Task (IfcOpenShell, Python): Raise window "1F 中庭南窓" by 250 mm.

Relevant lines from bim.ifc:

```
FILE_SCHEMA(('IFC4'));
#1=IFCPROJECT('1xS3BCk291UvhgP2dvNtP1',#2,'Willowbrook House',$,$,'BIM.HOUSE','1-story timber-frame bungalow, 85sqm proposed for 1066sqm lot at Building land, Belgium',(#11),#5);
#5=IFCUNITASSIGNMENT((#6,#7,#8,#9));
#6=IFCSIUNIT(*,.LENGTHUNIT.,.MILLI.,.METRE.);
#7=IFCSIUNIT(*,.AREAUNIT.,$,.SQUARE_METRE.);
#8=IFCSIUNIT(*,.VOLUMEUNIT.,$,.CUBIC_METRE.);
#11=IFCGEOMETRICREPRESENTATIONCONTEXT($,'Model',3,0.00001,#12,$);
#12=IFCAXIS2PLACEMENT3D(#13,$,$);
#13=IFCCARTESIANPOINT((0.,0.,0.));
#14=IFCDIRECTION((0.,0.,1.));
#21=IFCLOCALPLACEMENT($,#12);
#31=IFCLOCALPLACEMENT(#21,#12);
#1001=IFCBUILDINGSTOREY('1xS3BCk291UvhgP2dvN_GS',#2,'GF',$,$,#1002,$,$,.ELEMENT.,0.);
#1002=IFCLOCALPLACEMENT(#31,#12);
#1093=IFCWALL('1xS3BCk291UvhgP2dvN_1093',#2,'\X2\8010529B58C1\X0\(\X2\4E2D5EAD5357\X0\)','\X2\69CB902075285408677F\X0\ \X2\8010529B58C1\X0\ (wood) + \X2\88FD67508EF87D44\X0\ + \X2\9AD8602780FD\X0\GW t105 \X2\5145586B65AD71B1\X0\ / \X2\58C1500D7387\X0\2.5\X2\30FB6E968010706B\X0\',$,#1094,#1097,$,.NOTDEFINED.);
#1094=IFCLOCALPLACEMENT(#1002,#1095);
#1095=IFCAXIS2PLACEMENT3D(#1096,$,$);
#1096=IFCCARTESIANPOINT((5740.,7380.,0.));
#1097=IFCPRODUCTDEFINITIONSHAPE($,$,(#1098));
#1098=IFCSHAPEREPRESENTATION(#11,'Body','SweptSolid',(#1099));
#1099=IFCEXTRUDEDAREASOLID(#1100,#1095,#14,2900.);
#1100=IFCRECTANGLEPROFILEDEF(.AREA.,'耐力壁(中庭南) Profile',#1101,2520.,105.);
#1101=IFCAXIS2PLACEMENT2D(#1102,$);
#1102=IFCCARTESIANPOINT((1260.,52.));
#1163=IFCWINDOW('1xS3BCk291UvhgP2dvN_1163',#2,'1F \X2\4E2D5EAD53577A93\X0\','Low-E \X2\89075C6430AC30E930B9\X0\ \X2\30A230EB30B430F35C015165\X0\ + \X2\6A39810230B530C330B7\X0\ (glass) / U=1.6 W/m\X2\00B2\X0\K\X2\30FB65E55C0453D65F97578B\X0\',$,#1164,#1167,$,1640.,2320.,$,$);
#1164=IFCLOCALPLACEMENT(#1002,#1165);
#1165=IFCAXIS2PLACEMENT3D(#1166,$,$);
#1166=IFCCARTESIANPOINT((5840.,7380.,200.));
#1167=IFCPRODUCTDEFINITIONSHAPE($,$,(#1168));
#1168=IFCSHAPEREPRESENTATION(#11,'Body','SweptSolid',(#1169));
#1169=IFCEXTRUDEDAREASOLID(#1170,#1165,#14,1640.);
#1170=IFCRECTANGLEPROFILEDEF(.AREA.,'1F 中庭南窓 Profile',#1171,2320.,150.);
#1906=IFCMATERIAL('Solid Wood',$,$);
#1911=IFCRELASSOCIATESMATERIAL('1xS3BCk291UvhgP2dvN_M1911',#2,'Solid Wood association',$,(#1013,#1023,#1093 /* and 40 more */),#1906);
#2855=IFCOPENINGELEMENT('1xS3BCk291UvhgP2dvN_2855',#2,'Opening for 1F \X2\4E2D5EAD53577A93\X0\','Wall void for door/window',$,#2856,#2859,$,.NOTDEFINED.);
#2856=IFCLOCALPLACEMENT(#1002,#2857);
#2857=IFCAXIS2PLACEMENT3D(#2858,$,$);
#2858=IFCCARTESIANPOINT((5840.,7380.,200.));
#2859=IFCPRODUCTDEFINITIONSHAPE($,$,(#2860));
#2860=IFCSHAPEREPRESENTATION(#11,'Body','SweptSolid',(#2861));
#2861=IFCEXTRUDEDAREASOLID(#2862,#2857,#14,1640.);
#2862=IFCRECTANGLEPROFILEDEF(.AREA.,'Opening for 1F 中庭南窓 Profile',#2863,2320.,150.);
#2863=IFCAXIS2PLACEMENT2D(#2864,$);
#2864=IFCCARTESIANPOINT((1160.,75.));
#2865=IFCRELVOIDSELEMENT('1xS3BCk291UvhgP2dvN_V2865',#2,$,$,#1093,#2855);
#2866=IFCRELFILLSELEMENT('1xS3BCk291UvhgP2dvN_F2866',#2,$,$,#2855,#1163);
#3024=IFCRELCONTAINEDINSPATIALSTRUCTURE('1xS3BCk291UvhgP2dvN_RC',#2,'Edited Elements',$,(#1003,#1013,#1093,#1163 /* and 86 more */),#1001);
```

```python
import numpy as np
import ifcopenshell
import ifcopenshell.api.geometry
import ifcopenshell.util.placement
import ifcopenshell.util.unit

model = ifcopenshell.open("bim.ifc")
unit_scale = ifcopenshell.util.unit.calculate_unit_scale(model)

window = model.by_guid("1xS3BCk291UvhgP2dvN_1163")
opening = window.FillsVoids[0].RelatingOpeningElement
dz = 250.0

shift = np.array([0.0, 0.0, dz])
# The window is not placed relative to its opening, so move both.
for product in (opening, window):
    matrix = ifcopenshell.util.placement.get_local_placement(product.ObjectPlacement)
    matrix[:3, 3] += shift
    ifcopenshell.api.geometry.edit_object_placement(model, product=product, matrix=matrix, is_si=False)

print(f"moved by {dz * unit_scale:+.3f} m")

model.write("bim_updated.ifc")
```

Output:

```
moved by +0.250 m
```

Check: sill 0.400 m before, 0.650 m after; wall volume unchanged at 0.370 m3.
